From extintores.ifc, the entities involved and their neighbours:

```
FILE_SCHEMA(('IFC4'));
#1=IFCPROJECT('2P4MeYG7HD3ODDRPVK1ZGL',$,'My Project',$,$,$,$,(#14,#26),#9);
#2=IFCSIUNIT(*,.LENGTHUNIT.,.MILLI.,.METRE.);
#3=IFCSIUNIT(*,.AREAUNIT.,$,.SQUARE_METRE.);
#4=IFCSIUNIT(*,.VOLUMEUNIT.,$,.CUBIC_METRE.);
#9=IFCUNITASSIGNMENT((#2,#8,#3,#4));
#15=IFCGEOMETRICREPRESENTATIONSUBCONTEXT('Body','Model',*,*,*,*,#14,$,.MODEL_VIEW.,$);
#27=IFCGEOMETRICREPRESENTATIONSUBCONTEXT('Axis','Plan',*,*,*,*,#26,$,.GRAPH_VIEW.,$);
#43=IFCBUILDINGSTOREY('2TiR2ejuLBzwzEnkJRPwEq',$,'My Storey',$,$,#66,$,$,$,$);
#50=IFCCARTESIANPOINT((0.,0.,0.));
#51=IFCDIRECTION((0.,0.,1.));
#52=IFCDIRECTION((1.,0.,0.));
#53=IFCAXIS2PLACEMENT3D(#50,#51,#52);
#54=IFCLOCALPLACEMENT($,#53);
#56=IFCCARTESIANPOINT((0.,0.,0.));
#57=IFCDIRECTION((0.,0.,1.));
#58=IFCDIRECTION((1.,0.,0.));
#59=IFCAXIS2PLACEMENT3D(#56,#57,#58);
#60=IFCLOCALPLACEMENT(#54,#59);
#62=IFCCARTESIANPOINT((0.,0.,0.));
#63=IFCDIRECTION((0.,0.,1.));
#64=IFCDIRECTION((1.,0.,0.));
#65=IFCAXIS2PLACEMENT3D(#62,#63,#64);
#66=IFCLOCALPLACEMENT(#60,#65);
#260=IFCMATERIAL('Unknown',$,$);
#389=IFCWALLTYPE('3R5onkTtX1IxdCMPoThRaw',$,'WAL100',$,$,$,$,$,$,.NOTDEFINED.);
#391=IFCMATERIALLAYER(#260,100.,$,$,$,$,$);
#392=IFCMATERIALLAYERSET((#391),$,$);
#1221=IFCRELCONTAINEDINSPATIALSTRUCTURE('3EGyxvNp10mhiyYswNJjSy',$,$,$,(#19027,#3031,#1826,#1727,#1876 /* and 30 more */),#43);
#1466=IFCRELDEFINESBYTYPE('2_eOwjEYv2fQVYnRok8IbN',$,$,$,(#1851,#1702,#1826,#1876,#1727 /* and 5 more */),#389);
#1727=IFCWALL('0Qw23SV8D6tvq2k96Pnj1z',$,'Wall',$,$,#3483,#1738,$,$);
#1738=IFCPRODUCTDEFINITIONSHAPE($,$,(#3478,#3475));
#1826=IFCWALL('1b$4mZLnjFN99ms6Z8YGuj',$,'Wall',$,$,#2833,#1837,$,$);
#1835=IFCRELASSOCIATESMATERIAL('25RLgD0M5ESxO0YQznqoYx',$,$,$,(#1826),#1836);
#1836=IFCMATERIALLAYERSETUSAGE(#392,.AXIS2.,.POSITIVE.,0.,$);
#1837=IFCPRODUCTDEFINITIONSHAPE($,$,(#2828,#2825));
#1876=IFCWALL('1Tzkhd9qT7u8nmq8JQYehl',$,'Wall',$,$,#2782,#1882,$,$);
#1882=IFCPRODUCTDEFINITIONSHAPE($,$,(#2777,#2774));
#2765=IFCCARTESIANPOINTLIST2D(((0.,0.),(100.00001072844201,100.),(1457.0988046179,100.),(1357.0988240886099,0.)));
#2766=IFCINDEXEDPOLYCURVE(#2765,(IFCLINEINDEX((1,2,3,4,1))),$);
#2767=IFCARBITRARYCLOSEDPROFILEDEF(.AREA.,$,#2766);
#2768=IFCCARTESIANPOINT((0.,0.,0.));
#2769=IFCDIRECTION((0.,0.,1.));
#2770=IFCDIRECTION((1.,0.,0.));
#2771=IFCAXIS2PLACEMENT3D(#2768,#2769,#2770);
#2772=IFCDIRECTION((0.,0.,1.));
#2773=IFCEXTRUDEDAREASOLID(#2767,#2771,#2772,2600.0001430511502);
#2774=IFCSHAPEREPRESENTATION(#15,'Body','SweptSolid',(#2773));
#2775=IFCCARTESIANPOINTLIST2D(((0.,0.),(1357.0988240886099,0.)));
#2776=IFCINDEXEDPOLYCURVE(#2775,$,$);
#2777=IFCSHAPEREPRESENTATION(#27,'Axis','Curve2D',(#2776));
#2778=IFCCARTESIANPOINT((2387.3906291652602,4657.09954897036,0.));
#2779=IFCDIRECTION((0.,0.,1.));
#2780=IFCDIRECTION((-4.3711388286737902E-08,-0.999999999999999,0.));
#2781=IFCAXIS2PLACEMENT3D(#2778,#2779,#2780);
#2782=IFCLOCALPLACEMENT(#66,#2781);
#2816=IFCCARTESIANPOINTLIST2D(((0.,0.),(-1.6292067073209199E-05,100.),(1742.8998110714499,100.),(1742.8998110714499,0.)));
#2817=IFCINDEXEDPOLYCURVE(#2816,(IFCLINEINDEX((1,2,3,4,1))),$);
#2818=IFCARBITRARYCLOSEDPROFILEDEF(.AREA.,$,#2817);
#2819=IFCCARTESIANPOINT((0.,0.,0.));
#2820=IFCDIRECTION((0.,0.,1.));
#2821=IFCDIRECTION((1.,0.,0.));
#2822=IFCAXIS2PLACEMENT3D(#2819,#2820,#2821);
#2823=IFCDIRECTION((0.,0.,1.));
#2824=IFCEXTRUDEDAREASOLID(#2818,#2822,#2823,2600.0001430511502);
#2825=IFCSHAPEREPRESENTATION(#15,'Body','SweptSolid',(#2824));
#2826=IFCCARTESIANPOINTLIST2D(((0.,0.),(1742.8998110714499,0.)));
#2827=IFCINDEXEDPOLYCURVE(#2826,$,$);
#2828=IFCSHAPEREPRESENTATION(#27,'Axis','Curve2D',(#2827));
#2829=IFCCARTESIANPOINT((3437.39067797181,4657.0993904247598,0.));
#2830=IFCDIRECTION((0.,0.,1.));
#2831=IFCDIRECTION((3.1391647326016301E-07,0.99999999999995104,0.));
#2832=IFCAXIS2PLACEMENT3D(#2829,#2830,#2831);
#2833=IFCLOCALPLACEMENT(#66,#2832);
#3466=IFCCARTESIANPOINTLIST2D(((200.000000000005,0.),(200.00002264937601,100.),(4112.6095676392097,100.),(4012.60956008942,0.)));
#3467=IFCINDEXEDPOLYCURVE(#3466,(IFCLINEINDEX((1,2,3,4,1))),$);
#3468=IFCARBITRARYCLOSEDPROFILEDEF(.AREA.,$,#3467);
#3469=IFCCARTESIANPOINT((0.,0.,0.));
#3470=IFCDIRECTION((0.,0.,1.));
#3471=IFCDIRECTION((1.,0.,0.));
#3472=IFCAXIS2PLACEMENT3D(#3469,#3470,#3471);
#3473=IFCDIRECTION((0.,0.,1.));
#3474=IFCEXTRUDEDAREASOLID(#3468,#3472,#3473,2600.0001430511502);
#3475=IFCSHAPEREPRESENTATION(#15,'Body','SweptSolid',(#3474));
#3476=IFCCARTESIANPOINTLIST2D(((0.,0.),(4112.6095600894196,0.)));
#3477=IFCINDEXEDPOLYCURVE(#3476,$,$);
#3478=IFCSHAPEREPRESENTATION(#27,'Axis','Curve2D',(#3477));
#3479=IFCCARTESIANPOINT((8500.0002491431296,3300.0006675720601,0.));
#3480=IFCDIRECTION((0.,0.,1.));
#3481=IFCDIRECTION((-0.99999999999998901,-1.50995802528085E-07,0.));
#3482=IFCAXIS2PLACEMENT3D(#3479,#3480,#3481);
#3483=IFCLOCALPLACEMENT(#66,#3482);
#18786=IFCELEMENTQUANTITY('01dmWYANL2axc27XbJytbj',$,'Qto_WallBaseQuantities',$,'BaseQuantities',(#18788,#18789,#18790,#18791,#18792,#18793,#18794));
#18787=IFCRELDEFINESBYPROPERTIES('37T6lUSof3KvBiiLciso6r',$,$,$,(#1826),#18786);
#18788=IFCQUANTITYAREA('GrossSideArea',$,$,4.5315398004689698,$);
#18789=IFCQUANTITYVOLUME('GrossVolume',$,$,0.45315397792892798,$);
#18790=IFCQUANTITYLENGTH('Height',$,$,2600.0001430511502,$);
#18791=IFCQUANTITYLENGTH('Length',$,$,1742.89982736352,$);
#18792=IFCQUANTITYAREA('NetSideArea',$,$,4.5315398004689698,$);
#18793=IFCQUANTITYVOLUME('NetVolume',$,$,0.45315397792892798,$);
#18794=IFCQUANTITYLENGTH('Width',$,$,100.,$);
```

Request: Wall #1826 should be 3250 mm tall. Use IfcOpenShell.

```python
import ifcopenshell
import ifcopenshell.api.pset
import ifcopenshell.geom
import ifcopenshell.util.element
import ifcopenshell.util.representation
import ifcopenshell.util.shape
import ifcopenshell.util.unit

model = ifcopenshell.open("extintores.ifc")
unit_scale = ifcopenshell.util.unit.calculate_unit_scale(model)
area_scale = ifcopenshell.util.unit.calculate_unit_scale(model, "AREAUNIT")
volume_scale = ifcopenshell.util.unit.calculate_unit_scale(model, "VOLUMEUNIT")
settings = ifcopenshell.geom.settings()


def volume(element):
    """Net volume in cubic metres, openings subtracted."""
    shape = ifcopenshell.geom.create_shape(settings, element)
    return ifcopenshell.util.shape.get_volume(shape.geometry)


wall = model.by_id(1826)
before = volume(wall)

body = ifcopenshell.util.representation.get_representation(wall, "Model", "Body")
solid = body.Items[0]
old_height = solid.Depth
solid.Depth = 3.25 / unit_scale
after = volume(wall)
thickness = 0.1  # wall thickness in metres

# Update the stored height, areas and volumes.
qto = model.by_id(ifcopenshell.util.element.get_pset(wall, "Qto_WallBaseQuantities", should_inherit=False)["id"])
ifcopenshell.api.pset.edit_qto(model, qto=qto, properties={
    "GrossSideArea": ifcopenshell.util.element.get_pset(wall, "Qto_WallBaseQuantities", "GrossSideArea") * solid.Depth / old_height,
    "GrossVolume": ifcopenshell.util.element.get_pset(wall, "Qto_WallBaseQuantities", "GrossVolume") * solid.Depth / old_height,
    "Height": solid.Depth,
    "NetSideArea": after / thickness / area_scale,
    "NetVolume": after / volume_scale,
})

print(f"height {old_height:g} -> {solid.Depth:g}, volume {before:.3f} -> {after:.3f} m3")

model.write("extintores_updated.ifc")
```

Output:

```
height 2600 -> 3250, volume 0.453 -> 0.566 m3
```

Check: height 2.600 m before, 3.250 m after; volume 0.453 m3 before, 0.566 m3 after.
